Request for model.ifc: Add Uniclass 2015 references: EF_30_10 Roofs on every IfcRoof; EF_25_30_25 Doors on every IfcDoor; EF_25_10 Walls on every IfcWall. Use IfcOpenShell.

First a look at what the model holds.

```python
import ifcopenshell

model = ifcopenshell.open("model.ifc")
print(model.schema)
print("classifications:", [c.Name for c in model.by_type("IfcClassification")])
for ifc_class in ("IfcDoor", "IfcRoof", "IfcStair", "IfcWall", "IfcWindow"):
    print(ifc_class, len(model.by_type(ifc_class)))
```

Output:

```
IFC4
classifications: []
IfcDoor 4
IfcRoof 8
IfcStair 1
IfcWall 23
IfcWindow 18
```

```python
import ifcopenshell
import ifcopenshell.api.classification

model = ifcopenshell.open("model.ifc")

system = ifcopenshell.api.classification.add_classification(model, classification="Uniclass 2015")

codes = {
    "IfcRoof": ("EF_30_10", "Roofs"),
    "IfcDoor": ("EF_25_30_25", "Doors"),
    "IfcWall": ("EF_25_10", "Walls"),
}
for ifc_class, (code, name) in codes.items():
    products = model.by_type(ifc_class)
    ifcopenshell.api.classification.add_reference(
        model, products=products, classification=system, identification=code, name=name
    )
    print(code, len(products))

model.write("model_updated.ifc")
```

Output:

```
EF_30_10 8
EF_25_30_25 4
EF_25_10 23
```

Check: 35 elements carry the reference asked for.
